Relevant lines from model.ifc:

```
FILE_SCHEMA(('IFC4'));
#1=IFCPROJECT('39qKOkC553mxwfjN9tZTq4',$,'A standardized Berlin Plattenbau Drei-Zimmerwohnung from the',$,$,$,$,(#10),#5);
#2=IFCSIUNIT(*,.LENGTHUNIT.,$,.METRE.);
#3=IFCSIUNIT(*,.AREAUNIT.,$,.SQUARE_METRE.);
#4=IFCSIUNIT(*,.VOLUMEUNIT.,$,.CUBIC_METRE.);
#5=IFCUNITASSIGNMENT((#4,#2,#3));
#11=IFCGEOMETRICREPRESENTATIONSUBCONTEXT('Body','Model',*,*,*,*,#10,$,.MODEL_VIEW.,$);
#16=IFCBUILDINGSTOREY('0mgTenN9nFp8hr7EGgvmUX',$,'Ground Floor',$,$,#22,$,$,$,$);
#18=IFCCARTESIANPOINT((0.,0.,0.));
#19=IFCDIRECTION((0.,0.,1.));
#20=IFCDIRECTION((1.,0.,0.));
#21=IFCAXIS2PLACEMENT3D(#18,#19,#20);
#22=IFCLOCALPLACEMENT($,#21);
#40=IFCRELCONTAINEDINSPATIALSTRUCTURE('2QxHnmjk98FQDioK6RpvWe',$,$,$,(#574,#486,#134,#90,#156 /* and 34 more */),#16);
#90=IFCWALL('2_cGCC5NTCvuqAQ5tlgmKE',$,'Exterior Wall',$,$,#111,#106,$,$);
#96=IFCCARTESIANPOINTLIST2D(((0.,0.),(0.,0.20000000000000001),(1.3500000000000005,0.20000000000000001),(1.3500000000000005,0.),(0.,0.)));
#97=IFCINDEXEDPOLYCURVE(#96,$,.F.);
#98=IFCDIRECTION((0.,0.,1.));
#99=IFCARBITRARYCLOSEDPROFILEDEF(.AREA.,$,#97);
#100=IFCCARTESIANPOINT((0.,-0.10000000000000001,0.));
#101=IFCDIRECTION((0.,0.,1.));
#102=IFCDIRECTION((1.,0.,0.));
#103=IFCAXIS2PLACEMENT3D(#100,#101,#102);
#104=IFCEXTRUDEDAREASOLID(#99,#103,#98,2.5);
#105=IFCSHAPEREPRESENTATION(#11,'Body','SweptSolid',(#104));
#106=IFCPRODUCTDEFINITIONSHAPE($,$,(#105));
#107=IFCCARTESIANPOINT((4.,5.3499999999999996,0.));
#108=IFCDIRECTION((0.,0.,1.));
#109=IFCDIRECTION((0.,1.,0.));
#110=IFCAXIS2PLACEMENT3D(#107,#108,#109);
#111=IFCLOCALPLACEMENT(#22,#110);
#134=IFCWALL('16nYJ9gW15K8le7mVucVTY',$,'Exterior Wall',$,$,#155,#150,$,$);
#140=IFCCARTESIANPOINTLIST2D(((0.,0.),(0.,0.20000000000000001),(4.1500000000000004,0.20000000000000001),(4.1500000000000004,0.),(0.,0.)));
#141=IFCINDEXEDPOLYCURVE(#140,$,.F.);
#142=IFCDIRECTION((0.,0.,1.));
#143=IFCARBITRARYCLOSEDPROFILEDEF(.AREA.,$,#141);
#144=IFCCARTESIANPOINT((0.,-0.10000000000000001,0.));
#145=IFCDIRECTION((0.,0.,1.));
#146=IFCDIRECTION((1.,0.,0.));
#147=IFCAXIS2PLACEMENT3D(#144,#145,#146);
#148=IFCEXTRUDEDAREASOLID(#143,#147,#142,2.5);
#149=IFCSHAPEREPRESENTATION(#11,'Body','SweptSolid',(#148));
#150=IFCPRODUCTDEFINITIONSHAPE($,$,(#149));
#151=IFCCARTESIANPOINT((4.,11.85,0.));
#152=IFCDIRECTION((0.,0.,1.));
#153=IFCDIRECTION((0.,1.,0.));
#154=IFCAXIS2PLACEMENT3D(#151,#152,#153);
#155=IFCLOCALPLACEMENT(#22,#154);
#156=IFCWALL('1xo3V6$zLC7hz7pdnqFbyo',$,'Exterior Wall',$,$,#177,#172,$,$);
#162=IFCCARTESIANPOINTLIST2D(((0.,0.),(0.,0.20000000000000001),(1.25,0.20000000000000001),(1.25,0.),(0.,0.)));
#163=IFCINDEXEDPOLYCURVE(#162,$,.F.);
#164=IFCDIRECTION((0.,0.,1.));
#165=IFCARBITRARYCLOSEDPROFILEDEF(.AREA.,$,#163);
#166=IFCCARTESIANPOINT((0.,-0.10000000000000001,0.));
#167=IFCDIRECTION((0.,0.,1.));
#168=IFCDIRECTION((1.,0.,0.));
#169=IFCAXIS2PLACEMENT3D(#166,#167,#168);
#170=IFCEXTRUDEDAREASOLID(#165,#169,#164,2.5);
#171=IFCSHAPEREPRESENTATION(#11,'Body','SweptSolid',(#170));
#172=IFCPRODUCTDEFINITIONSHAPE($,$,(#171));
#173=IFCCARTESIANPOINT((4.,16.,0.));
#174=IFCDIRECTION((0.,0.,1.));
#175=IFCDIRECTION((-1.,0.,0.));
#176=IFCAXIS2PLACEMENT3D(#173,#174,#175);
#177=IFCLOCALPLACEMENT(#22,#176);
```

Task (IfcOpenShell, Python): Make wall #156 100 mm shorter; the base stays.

```python
import ifcopenshell
import ifcopenshell.geom
import ifcopenshell.util.representation
import ifcopenshell.util.shape

model = ifcopenshell.open("model.ifc")
settings = ifcopenshell.geom.settings()


def volume(element):
    """Net volume in cubic metres, openings subtracted."""
    shape = ifcopenshell.geom.create_shape(settings, element)
    return ifcopenshell.util.shape.get_volume(shape.geometry)


wall = model.by_guid("1xo3V6$zLC7hz7pdnqFbyo")
before = volume(wall)

body = ifcopenshell.util.representation.get_representation(wall, "Model", "Body")
solid = body.Items[0]
old_height = solid.Depth
solid.Depth -= 0.1
after = volume(wall)

print(f"height {old_height:g} -> {solid.Depth:g}, volume {before:.3f} -> {after:.3f} m3")

model.write("model_updated.ifc")
```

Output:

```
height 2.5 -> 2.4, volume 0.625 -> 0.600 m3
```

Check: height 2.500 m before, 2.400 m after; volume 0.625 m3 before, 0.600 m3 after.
